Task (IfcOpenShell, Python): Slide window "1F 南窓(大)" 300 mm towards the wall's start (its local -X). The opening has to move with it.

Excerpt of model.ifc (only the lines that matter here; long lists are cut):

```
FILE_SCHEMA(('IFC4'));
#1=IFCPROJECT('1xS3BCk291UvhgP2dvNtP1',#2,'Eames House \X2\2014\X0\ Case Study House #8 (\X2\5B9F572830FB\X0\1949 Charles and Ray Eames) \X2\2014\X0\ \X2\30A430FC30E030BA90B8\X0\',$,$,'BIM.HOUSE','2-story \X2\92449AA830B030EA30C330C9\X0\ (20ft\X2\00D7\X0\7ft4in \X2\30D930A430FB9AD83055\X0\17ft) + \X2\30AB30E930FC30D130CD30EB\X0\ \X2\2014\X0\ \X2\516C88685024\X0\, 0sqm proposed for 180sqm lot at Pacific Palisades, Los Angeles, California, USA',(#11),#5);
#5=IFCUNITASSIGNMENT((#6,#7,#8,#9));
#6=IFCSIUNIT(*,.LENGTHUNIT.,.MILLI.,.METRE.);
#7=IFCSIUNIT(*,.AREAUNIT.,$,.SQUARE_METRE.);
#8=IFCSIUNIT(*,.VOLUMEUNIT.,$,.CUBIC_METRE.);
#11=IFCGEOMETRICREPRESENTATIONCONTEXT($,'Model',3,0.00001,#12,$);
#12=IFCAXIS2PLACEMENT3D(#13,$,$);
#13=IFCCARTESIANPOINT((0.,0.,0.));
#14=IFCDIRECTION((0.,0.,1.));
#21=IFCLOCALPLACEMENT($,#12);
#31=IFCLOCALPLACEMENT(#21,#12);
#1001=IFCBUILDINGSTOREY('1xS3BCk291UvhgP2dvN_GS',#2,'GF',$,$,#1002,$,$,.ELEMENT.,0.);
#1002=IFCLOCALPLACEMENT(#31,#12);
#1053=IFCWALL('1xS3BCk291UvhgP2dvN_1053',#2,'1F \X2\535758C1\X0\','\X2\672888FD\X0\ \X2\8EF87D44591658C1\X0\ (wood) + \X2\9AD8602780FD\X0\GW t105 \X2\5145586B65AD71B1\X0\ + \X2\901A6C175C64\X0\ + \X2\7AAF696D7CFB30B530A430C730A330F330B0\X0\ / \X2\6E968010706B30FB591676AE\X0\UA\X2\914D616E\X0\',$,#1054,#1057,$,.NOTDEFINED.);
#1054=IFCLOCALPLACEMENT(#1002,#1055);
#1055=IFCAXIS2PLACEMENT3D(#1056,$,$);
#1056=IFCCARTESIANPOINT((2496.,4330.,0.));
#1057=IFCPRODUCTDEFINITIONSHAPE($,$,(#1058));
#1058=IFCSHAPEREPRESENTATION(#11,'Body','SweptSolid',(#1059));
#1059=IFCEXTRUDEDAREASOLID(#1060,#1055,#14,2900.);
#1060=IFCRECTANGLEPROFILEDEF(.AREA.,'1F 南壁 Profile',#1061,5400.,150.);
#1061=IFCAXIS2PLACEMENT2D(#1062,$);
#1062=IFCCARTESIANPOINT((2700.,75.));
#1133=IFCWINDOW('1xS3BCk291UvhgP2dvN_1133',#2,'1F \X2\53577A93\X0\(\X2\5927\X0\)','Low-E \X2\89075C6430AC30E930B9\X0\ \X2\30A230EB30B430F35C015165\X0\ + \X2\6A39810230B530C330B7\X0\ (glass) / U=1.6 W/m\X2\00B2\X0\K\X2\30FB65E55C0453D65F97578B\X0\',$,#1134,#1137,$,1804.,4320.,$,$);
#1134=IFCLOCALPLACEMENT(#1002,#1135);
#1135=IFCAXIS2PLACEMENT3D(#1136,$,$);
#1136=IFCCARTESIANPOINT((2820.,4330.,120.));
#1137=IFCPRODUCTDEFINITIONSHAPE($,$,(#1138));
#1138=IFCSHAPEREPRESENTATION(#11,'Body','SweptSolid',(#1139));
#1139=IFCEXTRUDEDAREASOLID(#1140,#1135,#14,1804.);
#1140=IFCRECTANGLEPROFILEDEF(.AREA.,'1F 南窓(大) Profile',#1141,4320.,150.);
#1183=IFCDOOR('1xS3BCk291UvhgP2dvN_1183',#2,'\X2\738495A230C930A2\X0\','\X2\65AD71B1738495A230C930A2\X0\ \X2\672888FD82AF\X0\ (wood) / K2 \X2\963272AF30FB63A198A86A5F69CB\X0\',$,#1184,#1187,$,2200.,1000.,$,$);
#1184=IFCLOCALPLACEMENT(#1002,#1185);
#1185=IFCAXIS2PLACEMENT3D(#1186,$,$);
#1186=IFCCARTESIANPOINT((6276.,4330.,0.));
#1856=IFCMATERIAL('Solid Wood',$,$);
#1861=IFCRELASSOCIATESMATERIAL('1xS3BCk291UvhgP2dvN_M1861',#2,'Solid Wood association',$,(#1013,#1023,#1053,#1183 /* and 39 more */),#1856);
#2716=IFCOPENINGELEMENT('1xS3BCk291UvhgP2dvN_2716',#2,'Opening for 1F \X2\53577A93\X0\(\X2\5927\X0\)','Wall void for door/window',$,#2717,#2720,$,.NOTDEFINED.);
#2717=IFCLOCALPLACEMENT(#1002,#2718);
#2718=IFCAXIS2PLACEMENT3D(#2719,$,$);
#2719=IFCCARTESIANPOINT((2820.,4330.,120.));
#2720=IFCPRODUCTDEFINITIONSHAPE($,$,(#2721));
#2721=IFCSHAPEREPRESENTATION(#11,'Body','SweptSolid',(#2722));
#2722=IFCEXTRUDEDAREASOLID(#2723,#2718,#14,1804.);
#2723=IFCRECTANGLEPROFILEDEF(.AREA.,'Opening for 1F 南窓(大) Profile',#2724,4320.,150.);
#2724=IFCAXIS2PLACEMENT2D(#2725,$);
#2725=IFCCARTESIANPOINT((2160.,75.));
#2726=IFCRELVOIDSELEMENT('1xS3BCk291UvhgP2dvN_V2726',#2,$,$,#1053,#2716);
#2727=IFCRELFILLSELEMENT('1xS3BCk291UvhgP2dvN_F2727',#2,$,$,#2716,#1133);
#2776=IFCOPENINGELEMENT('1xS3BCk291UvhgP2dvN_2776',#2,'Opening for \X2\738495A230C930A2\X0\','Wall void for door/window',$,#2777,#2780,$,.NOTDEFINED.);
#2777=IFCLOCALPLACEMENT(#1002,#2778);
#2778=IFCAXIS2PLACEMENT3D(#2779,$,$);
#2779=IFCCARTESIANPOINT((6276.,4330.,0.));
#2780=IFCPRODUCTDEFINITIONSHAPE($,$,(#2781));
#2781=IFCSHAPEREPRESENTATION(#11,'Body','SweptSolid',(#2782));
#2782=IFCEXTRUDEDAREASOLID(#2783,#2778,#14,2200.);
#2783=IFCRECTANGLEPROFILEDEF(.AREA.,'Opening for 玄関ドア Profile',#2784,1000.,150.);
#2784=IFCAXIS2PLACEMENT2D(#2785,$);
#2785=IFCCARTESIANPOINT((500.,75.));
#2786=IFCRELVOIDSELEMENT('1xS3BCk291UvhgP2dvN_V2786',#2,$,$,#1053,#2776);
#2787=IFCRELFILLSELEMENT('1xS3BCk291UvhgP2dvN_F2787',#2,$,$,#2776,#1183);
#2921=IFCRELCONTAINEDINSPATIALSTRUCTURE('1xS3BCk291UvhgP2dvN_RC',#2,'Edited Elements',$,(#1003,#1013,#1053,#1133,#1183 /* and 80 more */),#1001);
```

```python
import ifcopenshell
import ifcopenshell.api.geometry
import ifcopenshell.util.placement
import ifcopenshell.util.unit

model = ifcopenshell.open("model.ifc")
unit_scale = ifcopenshell.util.unit.calculate_unit_scale(model)

window = model.by_guid("1xS3BCk291UvhgP2dvN_1133")
opening = window.FillsVoids[0].RelatingOpeningElement
wall = opening.VoidsElements[0].RelatingBuildingElement

wall_matrix = ifcopenshell.util.placement.get_local_placement(wall.ObjectPlacement)
shift = wall_matrix[:3, 0] * -0.3 / unit_scale
before = ifcopenshell.util.placement.get_local_placement(window.ObjectPlacement)[:3, 3].copy()

# The window is not placed relative to its opening, so move both.
for product in (opening, window):
    matrix = ifcopenshell.util.placement.get_local_placement(product.ObjectPlacement)
    matrix[:3, 3] += shift
    ifcopenshell.api.geometry.edit_object_placement(model, product=product, matrix=matrix, is_si=False)

after = ifcopenshell.util.placement.get_local_placement(window.ObjectPlacement)[:3, 3]
print("window moved by", (after - before).round(3) + 0.0)

model.write("model_rev.ifc")
```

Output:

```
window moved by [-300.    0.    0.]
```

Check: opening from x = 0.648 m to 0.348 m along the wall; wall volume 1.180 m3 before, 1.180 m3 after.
